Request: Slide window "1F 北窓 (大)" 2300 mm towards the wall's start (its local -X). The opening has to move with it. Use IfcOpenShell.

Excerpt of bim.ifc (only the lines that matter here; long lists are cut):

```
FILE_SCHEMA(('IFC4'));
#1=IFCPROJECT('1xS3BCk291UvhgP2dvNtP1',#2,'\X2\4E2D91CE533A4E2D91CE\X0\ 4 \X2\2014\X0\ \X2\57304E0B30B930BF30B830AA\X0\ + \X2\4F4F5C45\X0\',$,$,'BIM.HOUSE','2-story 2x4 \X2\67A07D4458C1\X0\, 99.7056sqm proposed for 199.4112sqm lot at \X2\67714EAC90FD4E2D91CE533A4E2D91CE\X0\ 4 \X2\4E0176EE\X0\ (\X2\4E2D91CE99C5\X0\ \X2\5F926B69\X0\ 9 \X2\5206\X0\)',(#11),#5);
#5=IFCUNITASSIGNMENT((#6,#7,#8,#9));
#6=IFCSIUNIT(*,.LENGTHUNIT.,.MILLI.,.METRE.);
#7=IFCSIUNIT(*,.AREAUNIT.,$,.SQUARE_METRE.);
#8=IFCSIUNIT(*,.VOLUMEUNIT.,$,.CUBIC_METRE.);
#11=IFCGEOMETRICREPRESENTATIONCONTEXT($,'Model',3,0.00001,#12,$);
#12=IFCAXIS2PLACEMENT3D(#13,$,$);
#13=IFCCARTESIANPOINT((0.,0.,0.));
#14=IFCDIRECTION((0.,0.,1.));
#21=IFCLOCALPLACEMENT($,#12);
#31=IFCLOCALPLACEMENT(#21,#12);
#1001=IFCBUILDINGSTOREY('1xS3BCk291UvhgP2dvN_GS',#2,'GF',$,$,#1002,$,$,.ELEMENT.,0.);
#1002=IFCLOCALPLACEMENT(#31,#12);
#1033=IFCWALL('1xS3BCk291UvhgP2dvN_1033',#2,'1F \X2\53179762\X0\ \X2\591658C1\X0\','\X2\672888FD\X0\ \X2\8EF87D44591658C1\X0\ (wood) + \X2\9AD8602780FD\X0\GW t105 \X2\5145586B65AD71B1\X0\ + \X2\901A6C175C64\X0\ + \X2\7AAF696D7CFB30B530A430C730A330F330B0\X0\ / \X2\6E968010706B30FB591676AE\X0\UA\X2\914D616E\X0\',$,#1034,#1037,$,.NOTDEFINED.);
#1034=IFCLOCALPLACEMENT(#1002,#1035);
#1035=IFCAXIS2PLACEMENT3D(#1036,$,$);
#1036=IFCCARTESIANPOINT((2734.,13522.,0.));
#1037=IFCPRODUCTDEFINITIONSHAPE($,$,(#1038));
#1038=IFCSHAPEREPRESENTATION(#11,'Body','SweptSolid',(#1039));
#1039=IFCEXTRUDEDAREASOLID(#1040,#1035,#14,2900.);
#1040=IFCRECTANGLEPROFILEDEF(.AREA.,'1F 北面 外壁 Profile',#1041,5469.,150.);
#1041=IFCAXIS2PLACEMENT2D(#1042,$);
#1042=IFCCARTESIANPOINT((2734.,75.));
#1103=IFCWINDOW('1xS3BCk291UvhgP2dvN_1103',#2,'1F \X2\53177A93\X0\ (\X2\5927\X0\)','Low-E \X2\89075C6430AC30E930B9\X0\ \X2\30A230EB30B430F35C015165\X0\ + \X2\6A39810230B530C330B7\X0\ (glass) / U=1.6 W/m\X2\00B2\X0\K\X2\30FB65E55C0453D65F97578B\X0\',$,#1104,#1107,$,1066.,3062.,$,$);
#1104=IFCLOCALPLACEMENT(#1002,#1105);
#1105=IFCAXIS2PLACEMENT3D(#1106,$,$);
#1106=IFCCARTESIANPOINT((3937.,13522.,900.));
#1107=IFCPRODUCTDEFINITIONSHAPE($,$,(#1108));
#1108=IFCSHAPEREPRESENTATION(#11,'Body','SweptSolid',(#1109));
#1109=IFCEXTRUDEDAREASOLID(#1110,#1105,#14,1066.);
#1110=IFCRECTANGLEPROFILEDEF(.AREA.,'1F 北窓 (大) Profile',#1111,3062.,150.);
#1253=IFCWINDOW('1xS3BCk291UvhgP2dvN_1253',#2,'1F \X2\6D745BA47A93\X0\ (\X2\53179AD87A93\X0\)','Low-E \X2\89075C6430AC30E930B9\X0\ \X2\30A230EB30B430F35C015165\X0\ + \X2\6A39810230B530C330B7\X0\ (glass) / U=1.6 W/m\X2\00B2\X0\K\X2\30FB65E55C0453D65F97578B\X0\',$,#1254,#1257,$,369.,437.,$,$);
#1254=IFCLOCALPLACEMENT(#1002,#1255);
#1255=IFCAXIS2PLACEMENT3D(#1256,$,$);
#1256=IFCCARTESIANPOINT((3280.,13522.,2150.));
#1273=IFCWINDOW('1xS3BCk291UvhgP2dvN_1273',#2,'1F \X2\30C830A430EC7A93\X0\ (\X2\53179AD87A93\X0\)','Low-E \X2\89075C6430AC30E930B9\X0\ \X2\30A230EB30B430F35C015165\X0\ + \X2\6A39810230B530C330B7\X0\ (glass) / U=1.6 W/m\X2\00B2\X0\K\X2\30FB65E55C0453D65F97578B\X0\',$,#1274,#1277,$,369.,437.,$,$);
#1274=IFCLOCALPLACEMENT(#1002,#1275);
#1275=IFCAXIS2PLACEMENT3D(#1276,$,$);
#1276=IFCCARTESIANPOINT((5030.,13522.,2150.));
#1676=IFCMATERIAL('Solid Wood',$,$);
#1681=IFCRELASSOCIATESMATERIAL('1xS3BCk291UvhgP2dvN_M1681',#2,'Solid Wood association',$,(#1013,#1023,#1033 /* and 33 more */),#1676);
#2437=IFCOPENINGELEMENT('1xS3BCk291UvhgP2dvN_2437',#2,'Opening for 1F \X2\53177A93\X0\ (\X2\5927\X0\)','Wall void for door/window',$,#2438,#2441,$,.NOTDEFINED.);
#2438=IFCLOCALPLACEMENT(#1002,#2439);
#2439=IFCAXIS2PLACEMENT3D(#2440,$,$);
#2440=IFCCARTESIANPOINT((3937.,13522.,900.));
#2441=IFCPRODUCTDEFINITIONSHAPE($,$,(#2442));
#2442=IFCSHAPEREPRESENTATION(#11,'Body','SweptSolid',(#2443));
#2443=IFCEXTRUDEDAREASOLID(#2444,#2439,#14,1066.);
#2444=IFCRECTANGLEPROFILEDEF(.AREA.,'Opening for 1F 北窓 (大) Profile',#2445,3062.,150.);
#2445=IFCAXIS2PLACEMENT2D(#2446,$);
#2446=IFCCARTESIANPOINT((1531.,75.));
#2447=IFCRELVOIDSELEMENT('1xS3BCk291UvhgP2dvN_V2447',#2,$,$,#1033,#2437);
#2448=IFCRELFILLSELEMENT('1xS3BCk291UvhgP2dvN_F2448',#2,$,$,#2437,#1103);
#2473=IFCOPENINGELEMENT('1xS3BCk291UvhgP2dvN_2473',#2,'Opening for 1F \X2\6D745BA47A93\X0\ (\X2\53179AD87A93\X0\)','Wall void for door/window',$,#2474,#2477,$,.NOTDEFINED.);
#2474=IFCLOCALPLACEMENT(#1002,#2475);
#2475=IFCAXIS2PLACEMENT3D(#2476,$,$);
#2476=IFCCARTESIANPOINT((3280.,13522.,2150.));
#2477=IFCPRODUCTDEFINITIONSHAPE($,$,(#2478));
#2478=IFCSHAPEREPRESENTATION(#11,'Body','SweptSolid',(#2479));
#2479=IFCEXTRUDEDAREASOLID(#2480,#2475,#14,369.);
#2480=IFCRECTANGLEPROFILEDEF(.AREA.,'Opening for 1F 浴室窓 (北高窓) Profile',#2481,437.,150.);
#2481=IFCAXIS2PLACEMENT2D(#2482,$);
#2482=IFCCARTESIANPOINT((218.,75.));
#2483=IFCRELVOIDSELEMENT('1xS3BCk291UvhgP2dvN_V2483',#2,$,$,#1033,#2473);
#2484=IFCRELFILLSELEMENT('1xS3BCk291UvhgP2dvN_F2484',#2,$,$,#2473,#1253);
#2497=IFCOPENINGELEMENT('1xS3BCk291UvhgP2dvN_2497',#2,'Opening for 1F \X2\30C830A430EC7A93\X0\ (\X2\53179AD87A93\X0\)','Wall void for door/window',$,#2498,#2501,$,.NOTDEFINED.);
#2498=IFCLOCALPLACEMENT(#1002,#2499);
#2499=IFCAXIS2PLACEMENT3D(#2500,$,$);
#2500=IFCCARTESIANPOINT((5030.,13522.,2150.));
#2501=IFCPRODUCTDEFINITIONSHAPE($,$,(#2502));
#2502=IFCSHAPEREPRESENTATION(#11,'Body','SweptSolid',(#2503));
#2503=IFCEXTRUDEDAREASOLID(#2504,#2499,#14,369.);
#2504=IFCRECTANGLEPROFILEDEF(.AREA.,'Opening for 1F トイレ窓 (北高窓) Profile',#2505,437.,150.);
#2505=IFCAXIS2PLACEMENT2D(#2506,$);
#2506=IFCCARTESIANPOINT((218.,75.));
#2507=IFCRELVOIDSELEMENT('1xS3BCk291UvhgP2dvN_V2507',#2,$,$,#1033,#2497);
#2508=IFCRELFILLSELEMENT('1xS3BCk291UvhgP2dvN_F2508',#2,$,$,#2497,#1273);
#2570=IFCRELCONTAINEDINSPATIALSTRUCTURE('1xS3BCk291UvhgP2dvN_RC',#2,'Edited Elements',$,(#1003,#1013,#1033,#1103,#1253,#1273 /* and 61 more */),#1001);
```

```python
import ifcopenshell
import ifcopenshell.api.geometry
import ifcopenshell.util.placement

model = ifcopenshell.open("bim.ifc")

window = model.by_id(1103)
opening = window.FillsVoids[0].RelatingOpeningElement
wall = opening.VoidsElements[0].RelatingBuildingElement

wall_matrix = ifcopenshell.util.placement.get_local_placement(wall.ObjectPlacement)
shift = wall_matrix[:3, 0] * -2300.0
before = ifcopenshell.util.placement.get_local_placement(window.ObjectPlacement)[:3, 3].copy()

# The window is not placed relative to its opening, so move both.
for product in (opening, window):
    matrix = ifcopenshell.util.placement.get_local_placement(product.ObjectPlacement)
    matrix[:3, 3] += shift
    ifcopenshell.api.geometry.edit_object_placement(model, product=product, matrix=matrix, is_si=False)

after = ifcopenshell.util.placement.get_local_placement(window.ObjectPlacement)[:3, 3]
print("window moved by", (after - before).round(3) + 0.0)

model.write("bim_edited.ifc")
```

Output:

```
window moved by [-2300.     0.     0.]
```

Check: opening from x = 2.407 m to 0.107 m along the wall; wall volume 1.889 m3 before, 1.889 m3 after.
